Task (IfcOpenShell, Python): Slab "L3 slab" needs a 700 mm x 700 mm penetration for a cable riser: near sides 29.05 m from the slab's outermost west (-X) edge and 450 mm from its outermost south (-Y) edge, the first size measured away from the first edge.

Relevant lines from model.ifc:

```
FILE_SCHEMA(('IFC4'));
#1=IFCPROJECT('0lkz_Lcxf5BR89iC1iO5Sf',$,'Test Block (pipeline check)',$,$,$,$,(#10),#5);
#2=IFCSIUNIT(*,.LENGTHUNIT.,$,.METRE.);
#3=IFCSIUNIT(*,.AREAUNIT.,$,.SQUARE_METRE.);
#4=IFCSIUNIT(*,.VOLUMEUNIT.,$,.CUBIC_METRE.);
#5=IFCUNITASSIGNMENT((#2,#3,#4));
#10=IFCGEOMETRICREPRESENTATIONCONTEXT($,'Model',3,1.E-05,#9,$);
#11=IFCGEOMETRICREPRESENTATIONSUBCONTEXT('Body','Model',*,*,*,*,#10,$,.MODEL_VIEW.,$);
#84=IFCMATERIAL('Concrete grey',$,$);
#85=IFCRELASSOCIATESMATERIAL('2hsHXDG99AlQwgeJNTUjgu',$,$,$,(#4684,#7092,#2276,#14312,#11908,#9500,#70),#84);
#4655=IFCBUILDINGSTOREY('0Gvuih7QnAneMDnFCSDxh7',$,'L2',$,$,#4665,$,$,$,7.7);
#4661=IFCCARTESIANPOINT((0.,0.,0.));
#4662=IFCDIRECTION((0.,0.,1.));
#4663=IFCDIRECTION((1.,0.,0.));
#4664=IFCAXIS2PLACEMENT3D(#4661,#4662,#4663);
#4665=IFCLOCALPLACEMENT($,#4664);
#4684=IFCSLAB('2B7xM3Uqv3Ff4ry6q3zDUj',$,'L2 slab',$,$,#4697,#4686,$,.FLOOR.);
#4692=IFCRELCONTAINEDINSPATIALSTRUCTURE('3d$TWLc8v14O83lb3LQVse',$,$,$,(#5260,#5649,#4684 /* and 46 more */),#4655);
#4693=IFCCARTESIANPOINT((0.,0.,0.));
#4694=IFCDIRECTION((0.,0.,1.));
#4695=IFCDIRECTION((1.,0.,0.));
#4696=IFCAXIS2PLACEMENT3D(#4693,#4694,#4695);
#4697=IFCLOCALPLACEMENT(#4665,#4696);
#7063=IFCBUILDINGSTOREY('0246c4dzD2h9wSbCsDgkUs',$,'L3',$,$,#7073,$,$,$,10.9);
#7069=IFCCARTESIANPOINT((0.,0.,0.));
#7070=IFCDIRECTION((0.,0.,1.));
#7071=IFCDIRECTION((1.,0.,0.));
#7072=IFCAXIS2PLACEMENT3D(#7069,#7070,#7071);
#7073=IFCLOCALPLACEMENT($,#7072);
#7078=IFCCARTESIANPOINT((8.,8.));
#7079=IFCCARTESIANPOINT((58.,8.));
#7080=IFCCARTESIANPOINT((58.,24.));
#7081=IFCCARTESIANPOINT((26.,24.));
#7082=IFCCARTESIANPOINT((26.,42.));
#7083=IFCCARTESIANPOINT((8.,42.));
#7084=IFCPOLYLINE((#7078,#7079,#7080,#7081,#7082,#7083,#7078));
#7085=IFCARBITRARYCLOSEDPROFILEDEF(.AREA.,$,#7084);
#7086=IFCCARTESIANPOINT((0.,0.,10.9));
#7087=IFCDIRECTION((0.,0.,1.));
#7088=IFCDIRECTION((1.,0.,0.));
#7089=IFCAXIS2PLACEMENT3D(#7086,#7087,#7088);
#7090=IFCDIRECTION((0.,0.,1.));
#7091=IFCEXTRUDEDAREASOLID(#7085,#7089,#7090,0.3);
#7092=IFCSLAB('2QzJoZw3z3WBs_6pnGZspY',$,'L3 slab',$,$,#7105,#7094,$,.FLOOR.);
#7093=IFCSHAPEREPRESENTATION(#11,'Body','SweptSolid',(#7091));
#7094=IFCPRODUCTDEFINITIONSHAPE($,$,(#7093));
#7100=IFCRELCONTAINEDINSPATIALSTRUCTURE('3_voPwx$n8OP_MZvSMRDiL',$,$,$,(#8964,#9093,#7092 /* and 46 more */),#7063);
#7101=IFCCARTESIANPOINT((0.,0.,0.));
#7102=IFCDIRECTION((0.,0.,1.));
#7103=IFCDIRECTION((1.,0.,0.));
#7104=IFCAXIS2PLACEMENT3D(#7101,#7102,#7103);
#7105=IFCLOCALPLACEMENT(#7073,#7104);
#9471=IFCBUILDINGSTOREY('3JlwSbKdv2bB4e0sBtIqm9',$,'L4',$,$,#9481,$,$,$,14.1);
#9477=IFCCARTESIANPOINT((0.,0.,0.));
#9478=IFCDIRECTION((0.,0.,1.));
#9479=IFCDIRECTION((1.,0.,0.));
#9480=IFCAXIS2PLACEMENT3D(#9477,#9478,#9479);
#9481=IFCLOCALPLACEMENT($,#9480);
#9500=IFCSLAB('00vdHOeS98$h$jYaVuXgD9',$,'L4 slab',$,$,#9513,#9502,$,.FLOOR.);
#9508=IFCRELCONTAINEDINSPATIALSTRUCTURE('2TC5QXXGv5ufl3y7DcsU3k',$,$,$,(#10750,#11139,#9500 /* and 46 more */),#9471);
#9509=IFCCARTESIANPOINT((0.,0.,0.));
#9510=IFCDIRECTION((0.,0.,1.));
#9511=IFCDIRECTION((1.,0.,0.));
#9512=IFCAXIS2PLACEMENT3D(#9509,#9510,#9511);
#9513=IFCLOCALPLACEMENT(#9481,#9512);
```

```python
import numpy as np
import ifcopenshell
import ifcopenshell.api.feature
import ifcopenshell.api.geometry
import ifcopenshell.api.root
import ifcopenshell.geom
import ifcopenshell.util.placement
import ifcopenshell.util.representation
import ifcopenshell.util.shape
import ifcopenshell.util.unit

model = ifcopenshell.open("model.ifc")
unit_scale = ifcopenshell.util.unit.calculate_unit_scale(model)
settings = ifcopenshell.geom.settings()


def volume(element):
    """Net volume in cubic metres, openings subtracted."""
    shape = ifcopenshell.geom.create_shape(settings, element)
    return ifcopenshell.util.shape.get_volume(shape.geometry)


slab = model.by_id(7092)
before = volume(slab)

# Extent in the slab's own axes, in metres. The edges named are its -X and -Y sides.
slab_shape = ifcopenshell.geom.create_shape(settings, slab)
vertices = ifcopenshell.util.shape.get_vertices(slab_shape.geometry)
x_min, y_min, bottom = vertices.min(axis=0)
top = vertices[:, 2].max()

opening = ifcopenshell.api.root.create_entity(model, ifc_class="IfcOpeningElement", name="Cable riser opening", predefined_type="OPENING")
context = ifcopenshell.util.representation.get_context(model, "Model", "Body", "MODEL_VIEW")
width, depth = 0.7, 0.7
outline = [(0.0, 0.0), (width, 0.0), (width, depth), (0.0, depth), (0.0, 0.0)]
# Overshoot both faces by 50 mm so the cut is clean.
shape = ifcopenshell.api.geometry.add_slab_representation(
    model, context=context, depth=top - bottom + 0.1, polyline=outline
)
ifcopenshell.api.geometry.assign_representation(model, product=opening, representation=shape)

matrix = ifcopenshell.util.placement.get_local_placement(slab.ObjectPlacement)
matrix[:, 3] = matrix @ np.append(np.array([x_min + 29.05, y_min + 0.45, bottom - 0.05]) / unit_scale, 1.0)
ifcopenshell.api.geometry.edit_object_placement(model, product=opening, matrix=matrix, is_si=False)
ifcopenshell.api.feature.add_feature(model, feature=opening, element=slab)

after = volume(slab)

print(f"slab volume {before:.3f} -> {after:.3f} m3")

model.write("model_edited.ifc")
```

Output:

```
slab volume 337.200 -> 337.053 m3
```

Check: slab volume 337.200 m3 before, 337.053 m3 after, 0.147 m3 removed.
